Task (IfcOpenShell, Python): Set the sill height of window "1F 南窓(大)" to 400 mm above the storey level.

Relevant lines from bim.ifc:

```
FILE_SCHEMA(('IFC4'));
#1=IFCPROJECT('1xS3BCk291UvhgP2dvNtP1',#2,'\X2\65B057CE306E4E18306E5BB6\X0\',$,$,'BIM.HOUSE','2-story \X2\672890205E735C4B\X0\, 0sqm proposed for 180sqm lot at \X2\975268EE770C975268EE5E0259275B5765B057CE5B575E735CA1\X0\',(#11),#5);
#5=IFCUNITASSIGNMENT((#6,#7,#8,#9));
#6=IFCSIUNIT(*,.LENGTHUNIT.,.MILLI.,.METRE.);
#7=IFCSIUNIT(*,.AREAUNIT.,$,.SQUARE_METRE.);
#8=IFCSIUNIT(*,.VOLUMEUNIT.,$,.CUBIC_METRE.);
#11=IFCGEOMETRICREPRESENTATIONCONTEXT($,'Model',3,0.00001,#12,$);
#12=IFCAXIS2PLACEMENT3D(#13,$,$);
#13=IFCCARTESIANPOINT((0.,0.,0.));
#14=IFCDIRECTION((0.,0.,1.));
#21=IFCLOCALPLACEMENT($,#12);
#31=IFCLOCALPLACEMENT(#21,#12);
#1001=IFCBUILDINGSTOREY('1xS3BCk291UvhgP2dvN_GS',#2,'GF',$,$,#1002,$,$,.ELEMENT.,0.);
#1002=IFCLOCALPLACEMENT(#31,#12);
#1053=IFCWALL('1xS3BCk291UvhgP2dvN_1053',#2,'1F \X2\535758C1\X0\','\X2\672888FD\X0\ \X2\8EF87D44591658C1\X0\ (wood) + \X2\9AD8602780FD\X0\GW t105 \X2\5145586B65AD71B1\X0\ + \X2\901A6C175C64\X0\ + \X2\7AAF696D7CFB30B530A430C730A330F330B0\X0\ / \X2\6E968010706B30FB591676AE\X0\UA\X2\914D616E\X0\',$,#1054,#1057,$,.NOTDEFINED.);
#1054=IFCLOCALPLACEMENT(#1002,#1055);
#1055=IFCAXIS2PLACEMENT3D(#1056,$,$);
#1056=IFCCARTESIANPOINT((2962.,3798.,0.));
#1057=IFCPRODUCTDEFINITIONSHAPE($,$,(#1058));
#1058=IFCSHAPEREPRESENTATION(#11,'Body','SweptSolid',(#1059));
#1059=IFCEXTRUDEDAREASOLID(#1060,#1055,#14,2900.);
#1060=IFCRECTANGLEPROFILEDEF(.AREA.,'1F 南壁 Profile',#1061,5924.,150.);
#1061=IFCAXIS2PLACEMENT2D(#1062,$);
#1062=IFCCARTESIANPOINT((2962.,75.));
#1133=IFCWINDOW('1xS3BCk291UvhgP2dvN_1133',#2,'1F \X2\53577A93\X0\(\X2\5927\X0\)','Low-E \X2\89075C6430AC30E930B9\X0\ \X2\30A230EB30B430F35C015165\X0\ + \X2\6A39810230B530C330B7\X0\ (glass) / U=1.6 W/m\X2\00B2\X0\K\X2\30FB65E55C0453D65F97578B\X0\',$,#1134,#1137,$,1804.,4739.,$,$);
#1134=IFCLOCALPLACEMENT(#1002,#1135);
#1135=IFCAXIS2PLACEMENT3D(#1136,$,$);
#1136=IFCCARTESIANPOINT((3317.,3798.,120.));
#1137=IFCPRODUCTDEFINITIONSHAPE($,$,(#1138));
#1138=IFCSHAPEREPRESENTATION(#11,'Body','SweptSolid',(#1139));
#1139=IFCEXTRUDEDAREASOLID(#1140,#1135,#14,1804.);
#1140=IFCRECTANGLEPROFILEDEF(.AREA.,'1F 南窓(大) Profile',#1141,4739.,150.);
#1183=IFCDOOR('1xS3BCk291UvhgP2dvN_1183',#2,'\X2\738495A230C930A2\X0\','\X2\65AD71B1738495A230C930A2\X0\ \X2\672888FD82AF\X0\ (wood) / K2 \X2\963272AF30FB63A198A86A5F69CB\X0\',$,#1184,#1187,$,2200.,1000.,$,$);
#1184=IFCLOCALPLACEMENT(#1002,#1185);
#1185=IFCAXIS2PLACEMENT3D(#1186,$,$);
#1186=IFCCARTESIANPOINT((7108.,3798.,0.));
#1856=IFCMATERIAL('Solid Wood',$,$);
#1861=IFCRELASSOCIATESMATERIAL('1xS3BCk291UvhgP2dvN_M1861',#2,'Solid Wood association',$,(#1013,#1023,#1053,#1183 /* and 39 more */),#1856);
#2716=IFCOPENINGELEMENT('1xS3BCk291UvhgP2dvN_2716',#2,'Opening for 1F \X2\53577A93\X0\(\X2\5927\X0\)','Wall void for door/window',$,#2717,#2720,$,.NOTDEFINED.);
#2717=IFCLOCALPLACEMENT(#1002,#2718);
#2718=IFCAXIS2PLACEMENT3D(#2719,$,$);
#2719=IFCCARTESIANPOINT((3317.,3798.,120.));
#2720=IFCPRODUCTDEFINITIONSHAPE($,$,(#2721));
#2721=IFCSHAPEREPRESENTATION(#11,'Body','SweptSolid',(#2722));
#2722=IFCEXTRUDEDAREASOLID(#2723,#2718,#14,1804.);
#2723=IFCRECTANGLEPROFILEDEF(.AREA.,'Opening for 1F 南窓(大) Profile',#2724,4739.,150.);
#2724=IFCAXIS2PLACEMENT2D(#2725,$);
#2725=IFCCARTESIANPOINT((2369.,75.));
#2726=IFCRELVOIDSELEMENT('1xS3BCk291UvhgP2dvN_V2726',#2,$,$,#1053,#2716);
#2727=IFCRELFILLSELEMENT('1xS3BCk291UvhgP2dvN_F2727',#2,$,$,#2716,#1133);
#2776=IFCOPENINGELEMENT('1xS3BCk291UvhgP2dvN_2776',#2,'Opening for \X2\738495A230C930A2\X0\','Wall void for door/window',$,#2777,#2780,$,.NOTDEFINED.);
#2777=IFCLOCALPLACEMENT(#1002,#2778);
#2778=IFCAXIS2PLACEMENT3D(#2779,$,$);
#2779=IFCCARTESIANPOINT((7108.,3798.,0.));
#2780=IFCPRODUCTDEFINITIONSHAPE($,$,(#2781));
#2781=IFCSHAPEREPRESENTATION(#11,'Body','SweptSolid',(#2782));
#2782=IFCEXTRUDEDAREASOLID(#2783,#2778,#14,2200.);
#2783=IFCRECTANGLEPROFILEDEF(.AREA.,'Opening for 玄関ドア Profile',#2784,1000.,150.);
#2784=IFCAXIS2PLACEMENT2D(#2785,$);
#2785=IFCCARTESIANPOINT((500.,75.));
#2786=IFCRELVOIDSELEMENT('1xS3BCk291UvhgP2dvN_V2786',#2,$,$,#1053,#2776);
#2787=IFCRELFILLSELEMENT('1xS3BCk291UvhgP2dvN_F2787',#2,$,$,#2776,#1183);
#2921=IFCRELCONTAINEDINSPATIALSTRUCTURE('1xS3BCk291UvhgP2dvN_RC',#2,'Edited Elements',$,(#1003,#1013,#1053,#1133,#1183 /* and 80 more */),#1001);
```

```python
import numpy as np
import ifcopenshell
import ifcopenshell.api.geometry
import ifcopenshell.geom
import ifcopenshell.util.element
import ifcopenshell.util.placement
import ifcopenshell.util.shape
import ifcopenshell.util.unit

model = ifcopenshell.open("bim.ifc")
unit_scale = ifcopenshell.util.unit.calculate_unit_scale(model)

window = model.by_guid("1xS3BCk291UvhgP2dvN_1133")
opening = window.FillsVoids[0].RelatingOpeningElement
storey = ifcopenshell.util.element.get_container(window, ifc_class="IfcBuildingStorey")
level = ifcopenshell.util.placement.get_local_placement(storey.ObjectPlacement)[2, 3]

# The opening's origin need not be at the sill, so measure its lowest point.
shape = ifcopenshell.geom.create_shape(ifcopenshell.geom.settings(), opening)
bottom = ifcopenshell.util.shape.get_shape_bottom_elevation(shape, shape.geometry) / unit_scale
dz = level + 400.0 - bottom

shift = np.array([0.0, 0.0, dz])
# The window is not placed relative to its opening, so move both.
for product in (opening, window):
    matrix = ifcopenshell.util.placement.get_local_placement(product.ObjectPlacement)
    matrix[:3, 3] += shift
    ifcopenshell.api.geometry.edit_object_placement(model, product=product, matrix=matrix, is_si=False)

print(f"moved by {dz * unit_scale:+.3f} m")

model.write("bim_v2.ifc")
```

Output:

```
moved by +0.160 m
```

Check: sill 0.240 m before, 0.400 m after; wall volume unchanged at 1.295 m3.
